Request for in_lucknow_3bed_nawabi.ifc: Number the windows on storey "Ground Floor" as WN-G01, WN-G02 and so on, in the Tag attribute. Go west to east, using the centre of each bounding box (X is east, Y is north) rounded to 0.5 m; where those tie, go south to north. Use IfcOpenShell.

First a look at what the model holds.

```python
import ifcopenshell
import ifcopenshell.util.element
import ifcopenshell.util.placement

model = ifcopenshell.open("in_lucknow_3bed_nawabi.ifc")
print(model.schema)
storey = next(s for s in model.by_type("IfcBuildingStorey") if s.Name == "Ground Floor")
windows = [e for e in ifcopenshell.util.element.get_decomposition(storey) if e.is_a("IfcWindow")]
for e in sorted(windows, key=lambda e: e.id()):
    origin = ifcopenshell.util.placement.get_local_placement(e.ObjectPlacement)[:3, 3]
    print(e.id(), e.Tag, e.Name, origin.round(2) + 0.0, sep=" | ")
```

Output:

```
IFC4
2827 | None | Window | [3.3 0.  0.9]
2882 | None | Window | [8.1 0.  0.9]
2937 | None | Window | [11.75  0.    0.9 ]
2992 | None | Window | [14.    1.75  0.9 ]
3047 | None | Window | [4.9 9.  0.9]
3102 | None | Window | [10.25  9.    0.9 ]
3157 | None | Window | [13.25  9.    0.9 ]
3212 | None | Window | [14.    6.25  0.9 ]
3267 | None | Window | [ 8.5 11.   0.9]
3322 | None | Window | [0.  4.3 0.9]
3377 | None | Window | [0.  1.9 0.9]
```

```python
import ifcopenshell
import ifcopenshell.geom
import ifcopenshell.util.element
import ifcopenshell.util.shape

model = ifcopenshell.open("in_lucknow_3bed_nawabi.ifc")
settings = ifcopenshell.geom.settings()
settings.set("use-world-coords", True)


def centre(element):
    shape = ifcopenshell.geom.create_shape(settings, element)
    return ifcopenshell.util.shape.get_bbox_centroid(shape.geometry)


storey = next(s for s in model.by_type("IfcBuildingStorey") if s.Name == "Ground Floor")
windows = [e for e in ifcopenshell.util.element.get_decomposition(storey) if e.is_a("IfcWindow")]

# Insertion points can sit at a corner or the storey origin, so sort by the geometry (in metres).
centres = {e: centre(e) for e in windows}
windows.sort(key=lambda e: (round(centres[e][0] / 0.5), centres[e][1]))

for i, e in enumerate(windows, start=1):
    number = f"WN-G{i:02d}"
    e.Tag = number
    print(e.id(), number)

model.write("in_lucknow_3bed_nawabi_rev.ifc")
```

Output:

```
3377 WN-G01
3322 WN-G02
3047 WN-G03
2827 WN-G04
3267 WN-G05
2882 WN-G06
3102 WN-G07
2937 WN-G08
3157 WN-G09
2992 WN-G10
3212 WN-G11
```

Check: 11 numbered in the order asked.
